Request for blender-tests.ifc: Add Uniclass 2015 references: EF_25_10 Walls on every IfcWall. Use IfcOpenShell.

First a look at what the model holds.

```python
import ifcopenshell

model = ifcopenshell.open("blender-tests.ifc")
print(model.schema)
print("classifications:", [c.Name for c in model.by_type("IfcClassification")])
for ifc_class in ("IfcDoor", "IfcRoof", "IfcStair", "IfcWall", "IfcWindow"):
    print(ifc_class, len(model.by_type(ifc_class)))
```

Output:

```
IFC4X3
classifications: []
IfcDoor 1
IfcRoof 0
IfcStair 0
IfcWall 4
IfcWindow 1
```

```python
import ifcopenshell
import ifcopenshell.api.classification

model = ifcopenshell.open("blender-tests.ifc")

system = ifcopenshell.api.classification.add_classification(model, classification="Uniclass 2015")

codes = {
    "IfcWall": ("EF_25_10", "Walls"),
}
for ifc_class, (code, name) in codes.items():
    products = model.by_type(ifc_class)
    ifcopenshell.api.classification.add_reference(
        model, products=products, classification=system, identification=code, name=name
    )
    print(code, len(products))

model.write("blender-tests_v2.ifc")
```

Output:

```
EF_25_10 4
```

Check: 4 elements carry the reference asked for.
